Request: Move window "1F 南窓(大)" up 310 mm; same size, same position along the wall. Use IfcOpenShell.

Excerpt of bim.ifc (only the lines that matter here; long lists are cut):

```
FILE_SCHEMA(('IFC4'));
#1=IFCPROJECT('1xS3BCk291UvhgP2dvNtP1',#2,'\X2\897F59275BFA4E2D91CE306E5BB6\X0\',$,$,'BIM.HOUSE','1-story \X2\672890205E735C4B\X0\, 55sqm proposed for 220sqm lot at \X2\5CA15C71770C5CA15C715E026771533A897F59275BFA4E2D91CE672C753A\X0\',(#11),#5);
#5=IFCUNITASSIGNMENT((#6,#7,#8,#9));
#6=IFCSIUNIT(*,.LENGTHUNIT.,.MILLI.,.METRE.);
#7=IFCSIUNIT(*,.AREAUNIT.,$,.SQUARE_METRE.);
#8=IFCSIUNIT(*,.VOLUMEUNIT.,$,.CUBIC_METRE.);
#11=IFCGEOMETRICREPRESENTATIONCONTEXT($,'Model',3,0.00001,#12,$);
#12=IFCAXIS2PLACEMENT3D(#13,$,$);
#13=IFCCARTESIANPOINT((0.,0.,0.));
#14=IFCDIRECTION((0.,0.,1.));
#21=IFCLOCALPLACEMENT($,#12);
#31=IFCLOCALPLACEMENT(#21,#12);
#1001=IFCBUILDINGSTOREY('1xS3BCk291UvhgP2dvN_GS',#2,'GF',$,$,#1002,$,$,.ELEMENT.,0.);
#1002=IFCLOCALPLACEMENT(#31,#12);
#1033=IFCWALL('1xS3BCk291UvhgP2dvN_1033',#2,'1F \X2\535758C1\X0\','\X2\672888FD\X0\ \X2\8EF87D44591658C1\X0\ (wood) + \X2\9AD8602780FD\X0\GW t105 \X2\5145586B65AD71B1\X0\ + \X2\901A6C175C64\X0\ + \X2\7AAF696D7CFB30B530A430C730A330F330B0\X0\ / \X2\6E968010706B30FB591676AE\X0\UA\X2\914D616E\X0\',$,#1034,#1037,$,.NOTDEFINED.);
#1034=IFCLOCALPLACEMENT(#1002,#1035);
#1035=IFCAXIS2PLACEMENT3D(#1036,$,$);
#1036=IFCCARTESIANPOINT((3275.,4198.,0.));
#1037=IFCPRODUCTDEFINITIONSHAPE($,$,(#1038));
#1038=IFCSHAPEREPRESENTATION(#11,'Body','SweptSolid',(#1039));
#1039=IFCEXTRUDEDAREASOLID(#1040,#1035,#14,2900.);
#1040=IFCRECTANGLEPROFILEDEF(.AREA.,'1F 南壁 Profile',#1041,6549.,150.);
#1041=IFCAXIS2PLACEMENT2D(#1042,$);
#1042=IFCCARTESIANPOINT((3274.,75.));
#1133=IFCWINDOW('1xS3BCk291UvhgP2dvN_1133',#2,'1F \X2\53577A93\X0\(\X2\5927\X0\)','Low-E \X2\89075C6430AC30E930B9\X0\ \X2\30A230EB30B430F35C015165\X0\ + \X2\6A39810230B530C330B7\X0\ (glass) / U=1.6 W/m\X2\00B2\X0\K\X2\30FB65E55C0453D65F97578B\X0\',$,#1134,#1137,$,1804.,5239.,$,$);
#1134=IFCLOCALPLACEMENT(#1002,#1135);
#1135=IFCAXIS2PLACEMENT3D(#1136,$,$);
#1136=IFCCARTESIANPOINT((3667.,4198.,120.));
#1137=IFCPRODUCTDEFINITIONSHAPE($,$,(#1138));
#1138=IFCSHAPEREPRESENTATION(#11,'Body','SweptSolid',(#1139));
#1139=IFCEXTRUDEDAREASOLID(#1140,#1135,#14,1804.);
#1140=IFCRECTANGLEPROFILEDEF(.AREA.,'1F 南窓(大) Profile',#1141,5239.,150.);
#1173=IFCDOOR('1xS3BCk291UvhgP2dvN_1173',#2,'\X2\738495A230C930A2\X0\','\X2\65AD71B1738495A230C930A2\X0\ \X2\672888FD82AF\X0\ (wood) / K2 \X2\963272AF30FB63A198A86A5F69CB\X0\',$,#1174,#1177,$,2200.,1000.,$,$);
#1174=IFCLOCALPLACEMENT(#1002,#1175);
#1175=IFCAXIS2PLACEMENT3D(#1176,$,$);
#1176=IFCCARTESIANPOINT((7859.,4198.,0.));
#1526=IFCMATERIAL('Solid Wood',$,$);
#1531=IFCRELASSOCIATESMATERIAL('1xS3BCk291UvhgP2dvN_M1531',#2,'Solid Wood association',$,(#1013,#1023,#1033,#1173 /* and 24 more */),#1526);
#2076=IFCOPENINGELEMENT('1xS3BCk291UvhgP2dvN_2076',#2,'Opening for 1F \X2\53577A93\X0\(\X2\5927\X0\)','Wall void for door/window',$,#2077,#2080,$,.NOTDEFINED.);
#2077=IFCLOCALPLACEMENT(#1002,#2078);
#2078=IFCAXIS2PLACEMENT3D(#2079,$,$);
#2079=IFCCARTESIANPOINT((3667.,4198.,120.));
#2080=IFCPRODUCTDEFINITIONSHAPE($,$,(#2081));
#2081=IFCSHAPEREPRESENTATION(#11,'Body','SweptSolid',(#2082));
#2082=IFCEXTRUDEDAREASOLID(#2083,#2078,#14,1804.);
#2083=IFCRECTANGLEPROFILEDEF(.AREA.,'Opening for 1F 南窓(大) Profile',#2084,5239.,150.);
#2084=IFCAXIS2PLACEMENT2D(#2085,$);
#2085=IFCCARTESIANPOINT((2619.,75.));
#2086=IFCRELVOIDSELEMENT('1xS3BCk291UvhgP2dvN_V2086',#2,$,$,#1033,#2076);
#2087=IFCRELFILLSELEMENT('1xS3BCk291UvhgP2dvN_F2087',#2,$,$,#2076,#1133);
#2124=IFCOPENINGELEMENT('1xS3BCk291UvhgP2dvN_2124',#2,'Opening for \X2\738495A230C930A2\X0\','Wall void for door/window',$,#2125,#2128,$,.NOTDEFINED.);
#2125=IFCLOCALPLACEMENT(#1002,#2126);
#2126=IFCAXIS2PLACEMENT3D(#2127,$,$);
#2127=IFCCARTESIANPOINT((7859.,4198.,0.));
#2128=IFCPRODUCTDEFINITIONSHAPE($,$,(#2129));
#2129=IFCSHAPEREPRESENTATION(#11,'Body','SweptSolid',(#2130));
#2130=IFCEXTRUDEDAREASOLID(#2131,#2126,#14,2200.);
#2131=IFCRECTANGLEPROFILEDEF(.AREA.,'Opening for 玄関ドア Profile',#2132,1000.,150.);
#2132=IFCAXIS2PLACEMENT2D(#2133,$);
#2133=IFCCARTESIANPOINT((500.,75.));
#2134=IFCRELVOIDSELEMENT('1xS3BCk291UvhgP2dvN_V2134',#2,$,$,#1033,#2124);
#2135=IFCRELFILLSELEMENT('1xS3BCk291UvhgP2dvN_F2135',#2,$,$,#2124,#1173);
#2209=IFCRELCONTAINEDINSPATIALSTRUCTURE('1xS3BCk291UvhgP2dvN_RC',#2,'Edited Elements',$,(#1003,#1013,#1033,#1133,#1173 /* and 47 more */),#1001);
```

```python
import numpy as np
import ifcopenshell
import ifcopenshell.api.geometry
import ifcopenshell.util.placement
import ifcopenshell.util.unit

model = ifcopenshell.open("bim.ifc")
unit_scale = ifcopenshell.util.unit.calculate_unit_scale(model)

window = model.by_id(1133)
opening = window.FillsVoids[0].RelatingOpeningElement
dz = 0.31 / unit_scale

shift = np.array([0.0, 0.0, dz])
# The window is not placed relative to its opening, so move both.
for product in (opening, window):
    matrix = ifcopenshell.util.placement.get_local_placement(product.ObjectPlacement)
    matrix[:3, 3] += shift
    ifcopenshell.api.geometry.edit_object_placement(model, product=product, matrix=matrix, is_si=False)

print(f"moved by {dz * unit_scale:+.3f} m")

model.write("bim_rev.ifc")
```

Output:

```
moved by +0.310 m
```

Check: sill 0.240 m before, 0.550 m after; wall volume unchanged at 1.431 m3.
